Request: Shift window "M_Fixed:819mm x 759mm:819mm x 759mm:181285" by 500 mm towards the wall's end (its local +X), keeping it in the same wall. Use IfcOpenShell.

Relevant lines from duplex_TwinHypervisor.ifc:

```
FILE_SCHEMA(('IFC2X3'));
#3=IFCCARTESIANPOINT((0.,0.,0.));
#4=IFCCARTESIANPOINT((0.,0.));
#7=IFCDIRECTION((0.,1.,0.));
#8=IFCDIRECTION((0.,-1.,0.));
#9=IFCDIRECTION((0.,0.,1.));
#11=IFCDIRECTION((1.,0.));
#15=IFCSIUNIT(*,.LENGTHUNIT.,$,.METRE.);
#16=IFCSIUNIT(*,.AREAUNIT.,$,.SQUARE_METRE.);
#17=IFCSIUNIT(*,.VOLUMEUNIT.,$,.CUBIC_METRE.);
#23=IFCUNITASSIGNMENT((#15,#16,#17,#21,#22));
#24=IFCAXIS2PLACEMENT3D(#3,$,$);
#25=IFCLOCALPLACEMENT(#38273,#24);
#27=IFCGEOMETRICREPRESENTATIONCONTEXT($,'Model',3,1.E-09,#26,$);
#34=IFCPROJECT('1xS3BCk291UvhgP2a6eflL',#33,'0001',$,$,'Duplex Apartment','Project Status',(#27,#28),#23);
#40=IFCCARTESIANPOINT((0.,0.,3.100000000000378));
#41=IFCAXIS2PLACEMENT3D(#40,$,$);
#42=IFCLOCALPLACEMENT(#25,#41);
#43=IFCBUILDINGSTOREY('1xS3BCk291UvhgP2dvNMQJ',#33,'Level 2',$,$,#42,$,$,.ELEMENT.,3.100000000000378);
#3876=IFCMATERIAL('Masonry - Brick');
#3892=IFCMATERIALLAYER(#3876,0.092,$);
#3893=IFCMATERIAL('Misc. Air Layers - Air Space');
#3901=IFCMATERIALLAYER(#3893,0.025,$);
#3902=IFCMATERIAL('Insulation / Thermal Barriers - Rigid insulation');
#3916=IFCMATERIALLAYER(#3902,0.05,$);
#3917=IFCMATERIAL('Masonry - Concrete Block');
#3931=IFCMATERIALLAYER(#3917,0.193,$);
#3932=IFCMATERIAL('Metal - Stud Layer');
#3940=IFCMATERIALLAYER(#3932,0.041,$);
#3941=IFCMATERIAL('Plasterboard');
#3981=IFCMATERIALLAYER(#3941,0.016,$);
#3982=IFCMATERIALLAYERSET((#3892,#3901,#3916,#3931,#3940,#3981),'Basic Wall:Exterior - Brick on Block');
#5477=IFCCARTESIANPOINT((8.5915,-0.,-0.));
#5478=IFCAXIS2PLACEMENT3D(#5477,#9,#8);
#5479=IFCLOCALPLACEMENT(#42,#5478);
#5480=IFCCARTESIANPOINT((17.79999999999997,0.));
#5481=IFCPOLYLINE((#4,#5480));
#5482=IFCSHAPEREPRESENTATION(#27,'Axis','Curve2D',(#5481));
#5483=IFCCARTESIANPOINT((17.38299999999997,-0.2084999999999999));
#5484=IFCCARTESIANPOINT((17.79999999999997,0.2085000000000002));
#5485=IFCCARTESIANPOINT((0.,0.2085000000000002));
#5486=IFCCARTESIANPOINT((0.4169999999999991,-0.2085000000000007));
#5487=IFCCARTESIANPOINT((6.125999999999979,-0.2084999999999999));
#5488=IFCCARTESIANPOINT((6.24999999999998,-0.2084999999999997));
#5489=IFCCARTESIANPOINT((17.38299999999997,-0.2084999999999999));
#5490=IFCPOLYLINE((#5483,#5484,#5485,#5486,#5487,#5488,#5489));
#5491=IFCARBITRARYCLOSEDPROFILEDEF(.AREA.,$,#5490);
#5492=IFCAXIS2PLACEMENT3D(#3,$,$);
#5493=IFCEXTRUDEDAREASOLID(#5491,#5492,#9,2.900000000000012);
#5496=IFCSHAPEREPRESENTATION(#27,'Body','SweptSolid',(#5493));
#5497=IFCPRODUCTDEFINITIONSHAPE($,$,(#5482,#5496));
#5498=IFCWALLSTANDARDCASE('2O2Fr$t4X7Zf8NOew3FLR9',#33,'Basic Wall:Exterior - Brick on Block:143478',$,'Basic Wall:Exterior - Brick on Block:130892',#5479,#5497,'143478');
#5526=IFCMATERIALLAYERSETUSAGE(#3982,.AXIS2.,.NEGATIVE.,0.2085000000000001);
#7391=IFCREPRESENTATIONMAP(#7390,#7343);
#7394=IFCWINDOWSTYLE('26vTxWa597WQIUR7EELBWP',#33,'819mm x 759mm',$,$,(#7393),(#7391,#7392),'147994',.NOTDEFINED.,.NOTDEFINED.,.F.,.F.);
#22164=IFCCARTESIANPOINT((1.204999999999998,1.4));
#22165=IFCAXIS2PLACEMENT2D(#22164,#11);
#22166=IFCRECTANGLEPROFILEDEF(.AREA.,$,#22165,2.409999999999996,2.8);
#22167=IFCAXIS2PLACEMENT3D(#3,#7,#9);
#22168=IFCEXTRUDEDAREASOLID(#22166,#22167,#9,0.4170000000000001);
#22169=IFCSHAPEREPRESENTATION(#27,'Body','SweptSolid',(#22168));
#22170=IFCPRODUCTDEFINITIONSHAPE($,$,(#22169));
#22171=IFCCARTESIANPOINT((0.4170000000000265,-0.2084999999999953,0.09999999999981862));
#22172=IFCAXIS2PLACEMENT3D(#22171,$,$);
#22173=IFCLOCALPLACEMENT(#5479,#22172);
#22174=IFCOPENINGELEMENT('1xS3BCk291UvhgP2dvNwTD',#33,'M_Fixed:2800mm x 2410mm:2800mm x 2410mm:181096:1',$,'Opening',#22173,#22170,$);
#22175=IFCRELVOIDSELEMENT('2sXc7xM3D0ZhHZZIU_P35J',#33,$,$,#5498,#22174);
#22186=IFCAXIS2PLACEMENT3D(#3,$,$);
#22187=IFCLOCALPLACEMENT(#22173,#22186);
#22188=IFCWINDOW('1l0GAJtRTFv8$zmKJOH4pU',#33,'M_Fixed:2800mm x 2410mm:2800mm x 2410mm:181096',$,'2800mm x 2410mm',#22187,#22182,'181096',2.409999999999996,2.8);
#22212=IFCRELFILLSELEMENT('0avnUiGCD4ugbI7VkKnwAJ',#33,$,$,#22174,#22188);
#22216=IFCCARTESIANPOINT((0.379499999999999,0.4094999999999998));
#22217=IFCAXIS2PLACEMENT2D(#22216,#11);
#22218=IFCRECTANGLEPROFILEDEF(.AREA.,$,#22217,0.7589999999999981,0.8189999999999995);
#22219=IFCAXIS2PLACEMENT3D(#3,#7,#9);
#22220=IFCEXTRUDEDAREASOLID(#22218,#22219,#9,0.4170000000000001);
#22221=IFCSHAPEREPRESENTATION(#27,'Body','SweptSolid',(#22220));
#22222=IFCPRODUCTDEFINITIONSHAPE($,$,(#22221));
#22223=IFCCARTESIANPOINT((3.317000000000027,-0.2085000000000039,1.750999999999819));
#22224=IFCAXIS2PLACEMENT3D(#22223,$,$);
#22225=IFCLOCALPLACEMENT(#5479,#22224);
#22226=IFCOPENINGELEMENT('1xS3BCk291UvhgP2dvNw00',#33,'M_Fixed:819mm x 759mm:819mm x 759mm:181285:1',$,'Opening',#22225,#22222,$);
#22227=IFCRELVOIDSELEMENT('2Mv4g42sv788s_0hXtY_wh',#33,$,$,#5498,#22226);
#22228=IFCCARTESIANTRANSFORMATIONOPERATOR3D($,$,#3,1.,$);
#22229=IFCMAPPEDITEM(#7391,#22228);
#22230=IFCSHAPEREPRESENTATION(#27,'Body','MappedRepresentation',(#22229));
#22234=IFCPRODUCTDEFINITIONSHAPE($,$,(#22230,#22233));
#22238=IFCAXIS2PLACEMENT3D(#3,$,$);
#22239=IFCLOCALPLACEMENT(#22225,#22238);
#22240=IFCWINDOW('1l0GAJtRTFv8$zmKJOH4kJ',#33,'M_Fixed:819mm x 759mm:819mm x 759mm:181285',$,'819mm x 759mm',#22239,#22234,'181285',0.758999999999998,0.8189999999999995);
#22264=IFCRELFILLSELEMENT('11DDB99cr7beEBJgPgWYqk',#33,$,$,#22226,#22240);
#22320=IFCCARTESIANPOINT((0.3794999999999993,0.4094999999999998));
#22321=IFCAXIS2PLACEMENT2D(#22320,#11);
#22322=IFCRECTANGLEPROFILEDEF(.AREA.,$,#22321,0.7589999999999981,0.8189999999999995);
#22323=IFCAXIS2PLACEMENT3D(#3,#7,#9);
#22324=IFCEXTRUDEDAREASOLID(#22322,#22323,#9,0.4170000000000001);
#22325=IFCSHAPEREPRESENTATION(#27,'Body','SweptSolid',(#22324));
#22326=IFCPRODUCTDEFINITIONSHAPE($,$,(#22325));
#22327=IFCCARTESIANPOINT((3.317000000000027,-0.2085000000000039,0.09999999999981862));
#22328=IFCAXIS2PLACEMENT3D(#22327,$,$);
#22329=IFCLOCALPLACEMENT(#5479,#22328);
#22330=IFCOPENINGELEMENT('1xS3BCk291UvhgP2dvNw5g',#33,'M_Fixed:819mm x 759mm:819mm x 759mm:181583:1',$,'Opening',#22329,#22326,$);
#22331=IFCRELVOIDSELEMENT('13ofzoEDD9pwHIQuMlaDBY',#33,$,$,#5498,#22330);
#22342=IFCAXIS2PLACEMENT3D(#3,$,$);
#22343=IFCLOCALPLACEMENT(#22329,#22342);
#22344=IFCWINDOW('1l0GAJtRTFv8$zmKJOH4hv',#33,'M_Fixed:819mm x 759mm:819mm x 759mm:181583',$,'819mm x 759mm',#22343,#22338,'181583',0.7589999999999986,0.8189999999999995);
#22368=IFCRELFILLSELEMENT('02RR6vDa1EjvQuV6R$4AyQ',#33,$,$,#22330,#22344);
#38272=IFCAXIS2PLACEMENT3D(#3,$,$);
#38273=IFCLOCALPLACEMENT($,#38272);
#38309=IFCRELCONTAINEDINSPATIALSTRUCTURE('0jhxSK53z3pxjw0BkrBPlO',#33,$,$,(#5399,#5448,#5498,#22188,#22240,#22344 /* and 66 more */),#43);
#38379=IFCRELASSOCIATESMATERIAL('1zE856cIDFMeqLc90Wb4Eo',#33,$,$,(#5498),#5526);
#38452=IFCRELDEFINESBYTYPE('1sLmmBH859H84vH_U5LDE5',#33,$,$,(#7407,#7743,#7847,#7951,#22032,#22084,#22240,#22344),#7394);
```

```python
import ifcopenshell
import ifcopenshell.api.geometry
import ifcopenshell.util.placement
import ifcopenshell.util.unit

model = ifcopenshell.open("duplex_TwinHypervisor.ifc")
unit_scale = ifcopenshell.util.unit.calculate_unit_scale(model)

window = model.by_guid("1l0GAJtRTFv8$zmKJOH4kJ")
opening = window.FillsVoids[0].RelatingOpeningElement
wall = opening.VoidsElements[0].RelatingBuildingElement

wall_matrix = ifcopenshell.util.placement.get_local_placement(wall.ObjectPlacement)
shift = wall_matrix[:3, 0] * 0.5 / unit_scale
before = ifcopenshell.util.placement.get_local_placement(window.ObjectPlacement)[:3, 3].copy()

# The window is placed relative to its opening, so it follows when the opening moves.
matrix = ifcopenshell.util.placement.get_local_placement(opening.ObjectPlacement)
matrix[:3, 3] += shift
ifcopenshell.api.geometry.edit_object_placement(
    model, product=opening, matrix=matrix, is_si=False, should_transform_children=True
)

after = ifcopenshell.util.placement.get_local_placement(window.ObjectPlacement)[:3, 3]
print("window moved by", (after - before).round(3) + 0.0)

model.write("duplex_TwinHypervisor_v2.ifc")
```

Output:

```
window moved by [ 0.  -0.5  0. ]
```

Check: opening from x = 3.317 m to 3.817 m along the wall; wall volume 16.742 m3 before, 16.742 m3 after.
